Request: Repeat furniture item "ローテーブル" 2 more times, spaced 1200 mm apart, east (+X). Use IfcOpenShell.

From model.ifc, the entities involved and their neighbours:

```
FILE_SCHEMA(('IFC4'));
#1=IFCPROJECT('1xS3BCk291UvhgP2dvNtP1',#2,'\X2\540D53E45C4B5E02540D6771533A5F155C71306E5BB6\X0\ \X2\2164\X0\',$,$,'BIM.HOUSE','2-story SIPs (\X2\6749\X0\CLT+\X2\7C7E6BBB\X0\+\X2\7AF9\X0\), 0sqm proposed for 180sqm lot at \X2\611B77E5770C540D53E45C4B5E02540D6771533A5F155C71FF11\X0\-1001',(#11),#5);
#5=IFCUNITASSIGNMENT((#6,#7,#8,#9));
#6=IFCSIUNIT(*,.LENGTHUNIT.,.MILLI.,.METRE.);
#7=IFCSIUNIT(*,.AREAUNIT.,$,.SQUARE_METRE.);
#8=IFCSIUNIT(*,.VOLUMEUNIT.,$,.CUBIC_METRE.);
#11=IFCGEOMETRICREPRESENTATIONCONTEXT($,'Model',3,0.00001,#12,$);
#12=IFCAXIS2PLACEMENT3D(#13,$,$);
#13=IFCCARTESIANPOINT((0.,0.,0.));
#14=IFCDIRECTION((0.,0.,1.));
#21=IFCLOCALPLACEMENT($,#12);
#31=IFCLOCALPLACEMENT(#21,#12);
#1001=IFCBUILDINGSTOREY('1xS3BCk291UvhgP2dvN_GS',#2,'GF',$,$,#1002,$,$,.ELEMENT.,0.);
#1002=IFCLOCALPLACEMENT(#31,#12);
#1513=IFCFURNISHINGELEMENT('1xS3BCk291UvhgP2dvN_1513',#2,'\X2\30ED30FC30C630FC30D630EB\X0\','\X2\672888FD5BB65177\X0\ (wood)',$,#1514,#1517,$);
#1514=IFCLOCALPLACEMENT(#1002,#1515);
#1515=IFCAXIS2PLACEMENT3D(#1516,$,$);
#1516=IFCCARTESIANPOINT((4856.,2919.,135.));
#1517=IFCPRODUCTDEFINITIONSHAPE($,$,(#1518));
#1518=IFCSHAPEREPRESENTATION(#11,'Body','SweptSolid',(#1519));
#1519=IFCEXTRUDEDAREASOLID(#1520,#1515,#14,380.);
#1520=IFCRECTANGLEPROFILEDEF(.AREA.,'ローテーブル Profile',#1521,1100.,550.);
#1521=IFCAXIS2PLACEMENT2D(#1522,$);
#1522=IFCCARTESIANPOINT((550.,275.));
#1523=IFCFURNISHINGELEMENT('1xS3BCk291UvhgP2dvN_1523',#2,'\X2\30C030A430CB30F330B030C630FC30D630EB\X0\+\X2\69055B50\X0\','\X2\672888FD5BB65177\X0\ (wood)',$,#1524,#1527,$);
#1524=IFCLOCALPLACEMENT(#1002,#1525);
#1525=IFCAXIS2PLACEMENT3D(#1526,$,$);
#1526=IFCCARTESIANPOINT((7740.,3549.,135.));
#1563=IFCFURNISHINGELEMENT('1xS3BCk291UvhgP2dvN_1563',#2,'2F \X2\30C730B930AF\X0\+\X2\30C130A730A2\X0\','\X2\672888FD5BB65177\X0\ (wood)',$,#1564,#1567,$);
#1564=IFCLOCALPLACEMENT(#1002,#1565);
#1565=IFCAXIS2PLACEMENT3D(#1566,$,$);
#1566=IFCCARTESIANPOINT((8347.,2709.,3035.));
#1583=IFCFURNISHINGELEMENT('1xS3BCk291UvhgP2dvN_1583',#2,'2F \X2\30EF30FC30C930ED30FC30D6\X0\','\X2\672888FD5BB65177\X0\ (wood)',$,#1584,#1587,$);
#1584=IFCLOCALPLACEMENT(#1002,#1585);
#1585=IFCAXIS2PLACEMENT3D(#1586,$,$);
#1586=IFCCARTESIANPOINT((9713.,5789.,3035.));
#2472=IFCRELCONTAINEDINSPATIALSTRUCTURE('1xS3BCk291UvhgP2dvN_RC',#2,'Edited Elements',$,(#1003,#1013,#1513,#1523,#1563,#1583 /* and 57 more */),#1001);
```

```python
import numpy as np
import ifcopenshell
import ifcopenshell.api.geometry
import ifcopenshell.api.root
import ifcopenshell.util.element
import ifcopenshell.util.placement
import ifcopenshell.util.unit

model = ifcopenshell.open("model.ifc")
unit_scale = ifcopenshell.util.unit.calculate_unit_scale(model)


def reuse_history(source, copy):
    """copy_class also copies each property set's owner history, people and application; keep the originals."""
    for rel in copy.IsDefinedBy:
        if rel.is_a("IfcRelDefinesByProperties") and (history := rel.RelatingPropertyDefinition.OwnerHistory):
            rel.RelatingPropertyDefinition.OwnerHistory = source.OwnerHistory
            ifcopenshell.util.element.remove_deep2(model, history)


source = model.by_guid("1xS3BCk291UvhgP2dvN_1513")
base = ifcopenshell.util.placement.get_local_placement(source.ObjectPlacement)
step = np.array([1.0, 0.0, 0.0]) * 1.2 / unit_scale

for i in range(1, 3):
    copy = ifcopenshell.api.root.copy_class(model, product=source)
    copy.Representation = ifcopenshell.util.element.copy_deep(
        model, source.Representation, exclude=["IfcGeometricRepresentationContext", "IfcRepresentationMap"]
    )
    reuse_history(source, copy)
    matrix = base.copy()
    matrix[:3, 3] += i * step
    print("added at", matrix[:3, 3].round(3) + 0.0)
    ifcopenshell.api.geometry.edit_object_placement(model, product=copy, matrix=matrix, is_si=False)

model.write("model_edited.ifc")
```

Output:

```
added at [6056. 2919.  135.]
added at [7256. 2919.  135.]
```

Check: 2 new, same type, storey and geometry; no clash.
